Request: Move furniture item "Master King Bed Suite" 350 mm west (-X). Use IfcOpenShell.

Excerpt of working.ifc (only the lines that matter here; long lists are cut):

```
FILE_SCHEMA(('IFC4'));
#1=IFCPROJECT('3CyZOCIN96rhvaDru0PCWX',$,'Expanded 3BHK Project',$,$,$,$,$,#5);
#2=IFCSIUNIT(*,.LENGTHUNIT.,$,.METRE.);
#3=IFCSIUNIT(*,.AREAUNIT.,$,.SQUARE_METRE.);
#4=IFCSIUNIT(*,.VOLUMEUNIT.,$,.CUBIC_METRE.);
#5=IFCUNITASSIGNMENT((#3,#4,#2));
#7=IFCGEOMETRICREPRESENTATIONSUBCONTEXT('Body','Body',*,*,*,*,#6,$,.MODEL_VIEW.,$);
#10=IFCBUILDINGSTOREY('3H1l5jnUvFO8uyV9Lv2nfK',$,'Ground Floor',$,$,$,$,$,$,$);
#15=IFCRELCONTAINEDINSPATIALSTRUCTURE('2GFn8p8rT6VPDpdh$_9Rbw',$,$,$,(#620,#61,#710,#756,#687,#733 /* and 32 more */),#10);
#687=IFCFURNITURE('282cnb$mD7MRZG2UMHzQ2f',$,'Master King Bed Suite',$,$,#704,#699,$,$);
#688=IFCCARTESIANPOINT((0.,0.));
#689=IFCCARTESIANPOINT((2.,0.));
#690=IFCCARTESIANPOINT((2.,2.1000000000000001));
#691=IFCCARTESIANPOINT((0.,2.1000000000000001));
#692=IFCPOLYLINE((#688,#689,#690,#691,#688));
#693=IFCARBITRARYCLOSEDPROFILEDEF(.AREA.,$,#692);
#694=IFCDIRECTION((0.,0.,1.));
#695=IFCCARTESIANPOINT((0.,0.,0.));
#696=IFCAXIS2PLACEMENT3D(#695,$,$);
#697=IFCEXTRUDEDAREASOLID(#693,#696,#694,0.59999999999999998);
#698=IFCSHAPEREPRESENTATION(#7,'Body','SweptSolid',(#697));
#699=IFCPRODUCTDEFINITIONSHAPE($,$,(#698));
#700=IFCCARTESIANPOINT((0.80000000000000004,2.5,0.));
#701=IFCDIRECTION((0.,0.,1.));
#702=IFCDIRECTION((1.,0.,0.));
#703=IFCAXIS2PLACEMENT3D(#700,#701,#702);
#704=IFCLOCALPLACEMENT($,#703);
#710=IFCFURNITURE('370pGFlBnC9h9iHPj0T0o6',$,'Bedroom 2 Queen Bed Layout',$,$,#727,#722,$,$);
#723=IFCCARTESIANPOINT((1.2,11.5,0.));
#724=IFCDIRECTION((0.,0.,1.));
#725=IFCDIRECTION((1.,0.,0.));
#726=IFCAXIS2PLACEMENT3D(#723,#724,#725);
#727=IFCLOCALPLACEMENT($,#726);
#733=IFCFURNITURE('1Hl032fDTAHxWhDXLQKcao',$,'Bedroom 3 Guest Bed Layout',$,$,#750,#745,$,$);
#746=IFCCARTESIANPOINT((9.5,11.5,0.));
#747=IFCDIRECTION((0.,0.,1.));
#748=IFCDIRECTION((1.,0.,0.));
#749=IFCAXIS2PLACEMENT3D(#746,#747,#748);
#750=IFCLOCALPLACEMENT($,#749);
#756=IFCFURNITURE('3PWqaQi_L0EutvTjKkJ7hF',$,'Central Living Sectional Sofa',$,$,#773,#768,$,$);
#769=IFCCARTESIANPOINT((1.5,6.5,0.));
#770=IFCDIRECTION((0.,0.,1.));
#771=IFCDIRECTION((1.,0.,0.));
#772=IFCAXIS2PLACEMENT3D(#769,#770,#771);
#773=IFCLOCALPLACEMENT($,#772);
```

```python
import ifcopenshell
import ifcopenshell.api.geometry
import ifcopenshell.util.placement
import ifcopenshell.util.unit

model = ifcopenshell.open("working.ifc")
unit_scale = ifcopenshell.util.unit.calculate_unit_scale(model)

item = model.by_guid("282cnb$mD7MRZG2UMHzQ2f")
matrix = ifcopenshell.util.placement.get_local_placement(item.ObjectPlacement)
matrix[0, 3] -= 0.35 / unit_scale
ifcopenshell.api.geometry.edit_object_placement(model, product=item, matrix=matrix, is_si=False)

print(ifcopenshell.util.placement.get_local_placement(item.ObjectPlacement).round(3) + 0.0)

model.write("working_edited.ifc")
```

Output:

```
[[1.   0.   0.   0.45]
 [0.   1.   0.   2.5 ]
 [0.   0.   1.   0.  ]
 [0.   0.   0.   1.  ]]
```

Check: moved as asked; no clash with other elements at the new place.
